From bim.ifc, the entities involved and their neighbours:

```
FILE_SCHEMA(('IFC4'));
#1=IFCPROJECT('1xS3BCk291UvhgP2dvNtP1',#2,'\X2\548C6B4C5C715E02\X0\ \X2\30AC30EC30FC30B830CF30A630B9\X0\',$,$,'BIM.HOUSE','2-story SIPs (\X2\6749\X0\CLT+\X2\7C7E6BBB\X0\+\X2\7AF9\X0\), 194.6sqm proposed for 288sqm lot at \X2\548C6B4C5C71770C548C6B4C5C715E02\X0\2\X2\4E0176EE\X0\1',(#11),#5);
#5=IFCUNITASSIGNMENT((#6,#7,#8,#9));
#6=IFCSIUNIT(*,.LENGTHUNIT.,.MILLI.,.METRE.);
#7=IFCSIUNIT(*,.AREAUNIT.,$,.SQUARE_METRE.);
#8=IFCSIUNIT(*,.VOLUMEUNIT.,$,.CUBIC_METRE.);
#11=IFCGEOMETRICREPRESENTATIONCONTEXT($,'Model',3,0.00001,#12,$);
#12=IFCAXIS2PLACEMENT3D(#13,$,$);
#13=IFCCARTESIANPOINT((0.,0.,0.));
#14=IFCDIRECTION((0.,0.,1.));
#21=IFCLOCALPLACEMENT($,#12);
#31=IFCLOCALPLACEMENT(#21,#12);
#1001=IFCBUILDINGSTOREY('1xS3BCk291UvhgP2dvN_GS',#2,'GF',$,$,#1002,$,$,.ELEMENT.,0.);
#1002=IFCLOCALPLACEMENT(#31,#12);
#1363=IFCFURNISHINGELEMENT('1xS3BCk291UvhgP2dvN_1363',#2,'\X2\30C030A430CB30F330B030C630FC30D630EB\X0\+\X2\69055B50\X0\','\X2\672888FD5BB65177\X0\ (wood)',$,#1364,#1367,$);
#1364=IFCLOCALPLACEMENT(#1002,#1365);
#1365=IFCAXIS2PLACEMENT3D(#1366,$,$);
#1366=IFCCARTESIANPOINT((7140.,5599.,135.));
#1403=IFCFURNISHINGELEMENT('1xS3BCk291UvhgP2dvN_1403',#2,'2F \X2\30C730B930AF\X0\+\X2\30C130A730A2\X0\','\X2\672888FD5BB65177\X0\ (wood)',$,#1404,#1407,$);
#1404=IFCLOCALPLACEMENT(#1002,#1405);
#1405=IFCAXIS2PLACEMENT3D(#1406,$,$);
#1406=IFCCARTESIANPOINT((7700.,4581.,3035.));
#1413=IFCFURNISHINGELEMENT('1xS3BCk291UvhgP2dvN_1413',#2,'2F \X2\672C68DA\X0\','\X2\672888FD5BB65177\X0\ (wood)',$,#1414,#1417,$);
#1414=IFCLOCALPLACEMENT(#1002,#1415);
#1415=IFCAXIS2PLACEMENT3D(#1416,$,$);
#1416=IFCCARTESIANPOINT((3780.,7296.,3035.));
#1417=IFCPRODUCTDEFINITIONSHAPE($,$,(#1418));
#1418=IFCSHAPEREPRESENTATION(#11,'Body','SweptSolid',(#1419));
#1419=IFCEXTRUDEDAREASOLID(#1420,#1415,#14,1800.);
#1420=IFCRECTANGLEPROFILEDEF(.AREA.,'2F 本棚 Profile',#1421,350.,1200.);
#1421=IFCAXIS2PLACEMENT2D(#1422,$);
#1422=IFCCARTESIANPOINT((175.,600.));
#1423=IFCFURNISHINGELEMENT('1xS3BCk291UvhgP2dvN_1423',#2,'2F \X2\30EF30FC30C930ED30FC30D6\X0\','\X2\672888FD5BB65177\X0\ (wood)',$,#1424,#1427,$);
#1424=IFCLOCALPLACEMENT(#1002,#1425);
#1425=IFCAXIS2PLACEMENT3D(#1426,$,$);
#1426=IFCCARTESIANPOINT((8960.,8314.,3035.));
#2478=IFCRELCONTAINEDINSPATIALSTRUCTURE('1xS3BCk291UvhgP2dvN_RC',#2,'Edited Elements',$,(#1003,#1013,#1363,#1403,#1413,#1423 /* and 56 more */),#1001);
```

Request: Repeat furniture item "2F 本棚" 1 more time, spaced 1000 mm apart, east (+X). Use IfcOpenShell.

```python
import numpy as np
import ifcopenshell
import ifcopenshell.api.geometry
import ifcopenshell.api.root
import ifcopenshell.util.element
import ifcopenshell.util.placement
import ifcopenshell.util.unit

model = ifcopenshell.open("bim.ifc")
unit_scale = ifcopenshell.util.unit.calculate_unit_scale(model)


def reuse_history(source, copy):
    """copy_class also copies each property set's owner history, people and application; keep the originals."""
    for rel in copy.IsDefinedBy:
        if rel.is_a("IfcRelDefinesByProperties") and (history := rel.RelatingPropertyDefinition.OwnerHistory):
            rel.RelatingPropertyDefinition.OwnerHistory = source.OwnerHistory
            ifcopenshell.util.element.remove_deep2(model, history)


source = model.by_id(1413)
base = ifcopenshell.util.placement.get_local_placement(source.ObjectPlacement)
step = np.array([1.0, 0.0, 0.0]) * 1 / unit_scale

for i in range(1, 2):
    copy = ifcopenshell.api.root.copy_class(model, product=source)
    copy.Representation = ifcopenshell.util.element.copy_deep(
        model, source.Representation, exclude=["IfcGeometricRepresentationContext", "IfcRepresentationMap"]
    )
    reuse_history(source, copy)
    matrix = base.copy()
    matrix[:3, 3] += i * step
    print("added at", matrix[:3, 3].round(3) + 0.0)
    ifcopenshell.api.geometry.edit_object_placement(model, product=copy, matrix=matrix, is_si=False)

model.write("bim-out.ifc")
```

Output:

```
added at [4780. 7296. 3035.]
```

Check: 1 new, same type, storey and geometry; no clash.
